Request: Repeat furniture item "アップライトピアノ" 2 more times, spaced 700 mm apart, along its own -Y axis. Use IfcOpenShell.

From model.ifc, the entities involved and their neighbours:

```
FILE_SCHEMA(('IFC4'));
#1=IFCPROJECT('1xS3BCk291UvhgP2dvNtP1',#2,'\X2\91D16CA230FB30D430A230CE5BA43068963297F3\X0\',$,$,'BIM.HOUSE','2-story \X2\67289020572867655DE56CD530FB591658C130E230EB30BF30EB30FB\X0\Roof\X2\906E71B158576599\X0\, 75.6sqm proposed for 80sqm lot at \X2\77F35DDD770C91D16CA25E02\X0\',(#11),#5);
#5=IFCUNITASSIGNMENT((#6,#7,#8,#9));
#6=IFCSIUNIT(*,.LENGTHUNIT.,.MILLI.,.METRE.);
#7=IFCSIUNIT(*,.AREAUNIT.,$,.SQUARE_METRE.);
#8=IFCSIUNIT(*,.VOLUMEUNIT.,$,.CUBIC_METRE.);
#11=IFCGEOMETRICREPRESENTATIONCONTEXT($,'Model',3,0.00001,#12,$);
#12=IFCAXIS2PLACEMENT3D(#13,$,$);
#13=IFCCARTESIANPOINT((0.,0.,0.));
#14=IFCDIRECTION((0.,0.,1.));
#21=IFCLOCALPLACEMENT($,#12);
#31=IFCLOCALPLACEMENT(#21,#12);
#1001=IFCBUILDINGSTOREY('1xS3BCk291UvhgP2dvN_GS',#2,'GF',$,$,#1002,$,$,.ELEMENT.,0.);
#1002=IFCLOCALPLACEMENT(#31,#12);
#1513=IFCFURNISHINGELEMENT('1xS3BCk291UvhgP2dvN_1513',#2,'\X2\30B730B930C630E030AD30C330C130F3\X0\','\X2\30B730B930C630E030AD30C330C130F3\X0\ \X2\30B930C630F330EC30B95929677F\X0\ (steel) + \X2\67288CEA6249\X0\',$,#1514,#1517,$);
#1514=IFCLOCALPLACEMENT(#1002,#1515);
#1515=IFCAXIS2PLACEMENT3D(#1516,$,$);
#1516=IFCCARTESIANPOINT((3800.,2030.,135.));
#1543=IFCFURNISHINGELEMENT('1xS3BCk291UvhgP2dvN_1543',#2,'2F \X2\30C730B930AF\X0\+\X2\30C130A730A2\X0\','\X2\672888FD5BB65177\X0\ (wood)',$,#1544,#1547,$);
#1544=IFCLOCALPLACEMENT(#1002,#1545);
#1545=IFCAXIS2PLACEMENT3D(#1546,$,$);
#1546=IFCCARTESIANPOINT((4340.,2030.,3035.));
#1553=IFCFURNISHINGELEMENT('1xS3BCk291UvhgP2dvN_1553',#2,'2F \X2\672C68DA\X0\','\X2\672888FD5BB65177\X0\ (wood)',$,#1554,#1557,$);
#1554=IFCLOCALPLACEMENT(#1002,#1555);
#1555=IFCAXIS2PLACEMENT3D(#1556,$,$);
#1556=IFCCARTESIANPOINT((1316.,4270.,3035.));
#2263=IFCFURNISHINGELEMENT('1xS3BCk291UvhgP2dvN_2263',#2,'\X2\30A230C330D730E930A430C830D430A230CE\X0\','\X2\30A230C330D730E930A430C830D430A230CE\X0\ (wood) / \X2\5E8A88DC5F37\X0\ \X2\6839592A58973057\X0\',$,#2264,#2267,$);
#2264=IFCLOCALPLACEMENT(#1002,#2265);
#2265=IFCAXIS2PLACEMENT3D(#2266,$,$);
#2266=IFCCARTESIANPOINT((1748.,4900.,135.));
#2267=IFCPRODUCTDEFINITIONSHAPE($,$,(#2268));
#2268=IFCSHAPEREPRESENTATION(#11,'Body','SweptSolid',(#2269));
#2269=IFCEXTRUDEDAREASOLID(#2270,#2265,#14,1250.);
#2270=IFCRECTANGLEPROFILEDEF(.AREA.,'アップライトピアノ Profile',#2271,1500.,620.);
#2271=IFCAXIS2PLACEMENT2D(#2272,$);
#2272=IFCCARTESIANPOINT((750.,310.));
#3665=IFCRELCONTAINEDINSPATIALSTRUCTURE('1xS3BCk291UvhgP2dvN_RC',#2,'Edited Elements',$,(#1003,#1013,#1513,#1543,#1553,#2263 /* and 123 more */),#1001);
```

```python
import ifcopenshell
import ifcopenshell.api.geometry
import ifcopenshell.api.root
import ifcopenshell.util.element
import ifcopenshell.util.placement
import ifcopenshell.util.unit

model = ifcopenshell.open("model.ifc")
unit_scale = ifcopenshell.util.unit.calculate_unit_scale(model)


def reuse_history(source, copy):
    """copy_class also copies each property set's owner history, people and application; keep the originals."""
    for rel in copy.IsDefinedBy:
        if rel.is_a("IfcRelDefinesByProperties") and (history := rel.RelatingPropertyDefinition.OwnerHistory):
            rel.RelatingPropertyDefinition.OwnerHistory = source.OwnerHistory
            ifcopenshell.util.element.remove_deep2(model, history)


source = model.by_guid("1xS3BCk291UvhgP2dvN_2263")
base = ifcopenshell.util.placement.get_local_placement(source.ObjectPlacement)
step = -base[:3, 1] * 0.7 / unit_scale

for i in range(1, 3):
    copy = ifcopenshell.api.root.copy_class(model, product=source)
    copy.Representation = ifcopenshell.util.element.copy_deep(
        model, source.Representation, exclude=["IfcGeometricRepresentationContext", "IfcRepresentationMap"]
    )
    reuse_history(source, copy)
    matrix = base.copy()
    matrix[:3, 3] += i * step
    print("added at", matrix[:3, 3].round(3) + 0.0)
    ifcopenshell.api.geometry.edit_object_placement(model, product=copy, matrix=matrix, is_si=False)

model.write("model_edited.ifc")
```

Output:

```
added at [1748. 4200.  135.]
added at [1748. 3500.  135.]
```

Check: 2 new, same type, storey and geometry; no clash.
